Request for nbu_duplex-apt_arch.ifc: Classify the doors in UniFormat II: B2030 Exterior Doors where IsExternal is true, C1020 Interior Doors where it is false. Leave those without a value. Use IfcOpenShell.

First a look at what the model holds.

```python
import ifcopenshell
import ifcopenshell.util.element

model = ifcopenshell.open("nbu_duplex-apt_arch.ifc")
print(model.schema)
print("classifications:", [c.Name for c in model.by_type("IfcClassification")])
values = [ifcopenshell.util.element.get_pset(e, "Pset_DoorCommon", "IsExternal") for e in model.by_type("IfcDoor")]
for value in (True, False, None):
    print("IsExternal", value, values.count(value))
```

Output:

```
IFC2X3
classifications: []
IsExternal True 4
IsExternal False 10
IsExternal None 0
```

```python
import ifcopenshell
import ifcopenshell.api.classification
import ifcopenshell.util.element

model = ifcopenshell.open("nbu_duplex-apt_arch.ifc")

# IFC2X3 requires Source and Edition and has no link from the project to the system.
system = model.create_entity("IfcClassification", Source="ASTM", Edition="E1557", Name="UniFormat II")

doors = model.by_type("IfcDoor")
external = {e: ifcopenshell.util.element.get_pset(e, "Pset_DoorCommon", "IsExternal") for e in doors}
for flag, code, name in ((True, "B2030", "Exterior Doors"), (False, "C1020", "Interior Doors")):
    products = [e for e in doors if external[e] is flag]
    ifcopenshell.api.classification.add_reference(
        model, products=products, classification=system, identification=code, name=name
    )
    print(code, len(products))

model.write("nbu_duplex-apt_arch_updated.ifc")
```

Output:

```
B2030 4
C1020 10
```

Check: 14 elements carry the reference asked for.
